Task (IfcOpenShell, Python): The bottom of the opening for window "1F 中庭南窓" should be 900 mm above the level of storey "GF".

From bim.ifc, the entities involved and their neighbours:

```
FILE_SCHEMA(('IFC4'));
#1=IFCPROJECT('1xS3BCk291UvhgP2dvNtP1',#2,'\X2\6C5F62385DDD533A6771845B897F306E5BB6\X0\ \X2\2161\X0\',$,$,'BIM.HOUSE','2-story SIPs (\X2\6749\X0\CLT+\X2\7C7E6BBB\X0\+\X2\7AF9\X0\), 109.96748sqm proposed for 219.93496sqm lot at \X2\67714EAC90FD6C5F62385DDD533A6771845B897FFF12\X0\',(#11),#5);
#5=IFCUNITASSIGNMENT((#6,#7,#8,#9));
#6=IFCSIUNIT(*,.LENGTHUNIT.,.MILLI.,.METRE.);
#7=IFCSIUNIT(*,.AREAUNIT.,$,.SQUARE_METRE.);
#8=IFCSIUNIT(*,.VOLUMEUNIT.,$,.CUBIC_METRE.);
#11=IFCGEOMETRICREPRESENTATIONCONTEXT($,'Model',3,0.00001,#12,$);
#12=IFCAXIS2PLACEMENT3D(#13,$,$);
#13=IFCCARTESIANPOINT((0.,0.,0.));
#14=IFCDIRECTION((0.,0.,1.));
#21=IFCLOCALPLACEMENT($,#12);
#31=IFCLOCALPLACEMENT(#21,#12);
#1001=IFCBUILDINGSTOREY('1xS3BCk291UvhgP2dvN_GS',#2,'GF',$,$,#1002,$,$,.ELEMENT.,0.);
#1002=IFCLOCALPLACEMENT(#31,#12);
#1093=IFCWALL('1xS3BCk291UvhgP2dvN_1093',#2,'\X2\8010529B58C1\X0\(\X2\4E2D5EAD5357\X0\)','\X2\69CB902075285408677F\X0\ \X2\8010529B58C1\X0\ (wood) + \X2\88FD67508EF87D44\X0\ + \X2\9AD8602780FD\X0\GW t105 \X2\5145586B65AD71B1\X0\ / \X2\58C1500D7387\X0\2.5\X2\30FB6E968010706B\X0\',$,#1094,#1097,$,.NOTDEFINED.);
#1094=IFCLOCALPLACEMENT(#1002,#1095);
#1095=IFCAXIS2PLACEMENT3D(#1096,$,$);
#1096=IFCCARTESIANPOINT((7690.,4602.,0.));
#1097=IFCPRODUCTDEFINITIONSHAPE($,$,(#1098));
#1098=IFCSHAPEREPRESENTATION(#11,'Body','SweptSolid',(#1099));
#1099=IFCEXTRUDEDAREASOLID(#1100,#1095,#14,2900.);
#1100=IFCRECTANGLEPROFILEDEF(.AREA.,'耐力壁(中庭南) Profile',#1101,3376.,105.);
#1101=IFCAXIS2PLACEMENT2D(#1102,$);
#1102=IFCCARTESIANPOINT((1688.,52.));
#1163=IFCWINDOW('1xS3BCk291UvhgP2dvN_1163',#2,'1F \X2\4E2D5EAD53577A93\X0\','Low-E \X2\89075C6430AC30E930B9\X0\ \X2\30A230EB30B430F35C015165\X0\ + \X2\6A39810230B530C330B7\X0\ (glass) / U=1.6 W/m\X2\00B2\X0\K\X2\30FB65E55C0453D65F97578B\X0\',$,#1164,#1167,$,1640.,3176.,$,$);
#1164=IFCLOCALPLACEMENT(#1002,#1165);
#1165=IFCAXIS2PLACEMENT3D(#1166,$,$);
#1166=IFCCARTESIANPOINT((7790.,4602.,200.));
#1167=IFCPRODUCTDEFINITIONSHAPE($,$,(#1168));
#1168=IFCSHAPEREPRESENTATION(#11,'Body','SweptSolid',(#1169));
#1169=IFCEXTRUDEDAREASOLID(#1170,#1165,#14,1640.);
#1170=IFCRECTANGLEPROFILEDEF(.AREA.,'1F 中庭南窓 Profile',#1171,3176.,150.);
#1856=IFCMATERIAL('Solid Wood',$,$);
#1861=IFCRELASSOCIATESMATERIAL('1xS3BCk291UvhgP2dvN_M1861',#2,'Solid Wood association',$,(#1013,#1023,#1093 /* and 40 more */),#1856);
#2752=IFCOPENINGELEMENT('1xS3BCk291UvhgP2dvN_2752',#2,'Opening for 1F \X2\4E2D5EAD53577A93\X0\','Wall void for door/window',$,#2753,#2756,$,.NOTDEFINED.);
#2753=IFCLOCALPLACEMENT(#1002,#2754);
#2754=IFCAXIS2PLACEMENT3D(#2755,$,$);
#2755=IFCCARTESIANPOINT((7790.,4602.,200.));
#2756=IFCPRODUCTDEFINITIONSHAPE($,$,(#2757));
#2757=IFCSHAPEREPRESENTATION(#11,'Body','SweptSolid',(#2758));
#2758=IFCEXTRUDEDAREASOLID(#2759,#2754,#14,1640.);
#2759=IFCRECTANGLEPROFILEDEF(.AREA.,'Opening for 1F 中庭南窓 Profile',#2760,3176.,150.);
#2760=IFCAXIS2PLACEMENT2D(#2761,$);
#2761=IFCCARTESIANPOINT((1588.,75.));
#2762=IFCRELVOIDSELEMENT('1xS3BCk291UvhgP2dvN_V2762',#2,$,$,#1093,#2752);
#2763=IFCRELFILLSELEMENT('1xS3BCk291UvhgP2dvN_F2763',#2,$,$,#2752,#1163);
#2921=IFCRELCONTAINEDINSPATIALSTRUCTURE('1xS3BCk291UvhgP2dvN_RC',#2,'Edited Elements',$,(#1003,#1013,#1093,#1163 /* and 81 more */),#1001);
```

```python
import numpy as np
import ifcopenshell
import ifcopenshell.api.geometry
import ifcopenshell.geom
import ifcopenshell.util.element
import ifcopenshell.util.placement
import ifcopenshell.util.shape
import ifcopenshell.util.unit

model = ifcopenshell.open("bim.ifc")
unit_scale = ifcopenshell.util.unit.calculate_unit_scale(model)

window = model.by_guid("1xS3BCk291UvhgP2dvN_1163")
opening = window.FillsVoids[0].RelatingOpeningElement
storey = ifcopenshell.util.element.get_container(window, ifc_class="IfcBuildingStorey")
level = ifcopenshell.util.placement.get_local_placement(storey.ObjectPlacement)[2, 3]

# The opening's origin need not be at the sill, so measure its lowest point.
shape = ifcopenshell.geom.create_shape(ifcopenshell.geom.settings(), opening)
bottom = ifcopenshell.util.shape.get_shape_bottom_elevation(shape, shape.geometry) / unit_scale
dz = level + 900.0 - bottom

shift = np.array([0.0, 0.0, dz])
# The window is not placed relative to its opening, so move both.
for product in (opening, window):
    matrix = ifcopenshell.util.placement.get_local_placement(product.ObjectPlacement)
    matrix[:3, 3] += shift
    ifcopenshell.api.geometry.edit_object_placement(model, product=product, matrix=matrix, is_si=False)

print(f"moved by {dz * unit_scale:+.3f} m")

model.write("bim-out.ifc")
```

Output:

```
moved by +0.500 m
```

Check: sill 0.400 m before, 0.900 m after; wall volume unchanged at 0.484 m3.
